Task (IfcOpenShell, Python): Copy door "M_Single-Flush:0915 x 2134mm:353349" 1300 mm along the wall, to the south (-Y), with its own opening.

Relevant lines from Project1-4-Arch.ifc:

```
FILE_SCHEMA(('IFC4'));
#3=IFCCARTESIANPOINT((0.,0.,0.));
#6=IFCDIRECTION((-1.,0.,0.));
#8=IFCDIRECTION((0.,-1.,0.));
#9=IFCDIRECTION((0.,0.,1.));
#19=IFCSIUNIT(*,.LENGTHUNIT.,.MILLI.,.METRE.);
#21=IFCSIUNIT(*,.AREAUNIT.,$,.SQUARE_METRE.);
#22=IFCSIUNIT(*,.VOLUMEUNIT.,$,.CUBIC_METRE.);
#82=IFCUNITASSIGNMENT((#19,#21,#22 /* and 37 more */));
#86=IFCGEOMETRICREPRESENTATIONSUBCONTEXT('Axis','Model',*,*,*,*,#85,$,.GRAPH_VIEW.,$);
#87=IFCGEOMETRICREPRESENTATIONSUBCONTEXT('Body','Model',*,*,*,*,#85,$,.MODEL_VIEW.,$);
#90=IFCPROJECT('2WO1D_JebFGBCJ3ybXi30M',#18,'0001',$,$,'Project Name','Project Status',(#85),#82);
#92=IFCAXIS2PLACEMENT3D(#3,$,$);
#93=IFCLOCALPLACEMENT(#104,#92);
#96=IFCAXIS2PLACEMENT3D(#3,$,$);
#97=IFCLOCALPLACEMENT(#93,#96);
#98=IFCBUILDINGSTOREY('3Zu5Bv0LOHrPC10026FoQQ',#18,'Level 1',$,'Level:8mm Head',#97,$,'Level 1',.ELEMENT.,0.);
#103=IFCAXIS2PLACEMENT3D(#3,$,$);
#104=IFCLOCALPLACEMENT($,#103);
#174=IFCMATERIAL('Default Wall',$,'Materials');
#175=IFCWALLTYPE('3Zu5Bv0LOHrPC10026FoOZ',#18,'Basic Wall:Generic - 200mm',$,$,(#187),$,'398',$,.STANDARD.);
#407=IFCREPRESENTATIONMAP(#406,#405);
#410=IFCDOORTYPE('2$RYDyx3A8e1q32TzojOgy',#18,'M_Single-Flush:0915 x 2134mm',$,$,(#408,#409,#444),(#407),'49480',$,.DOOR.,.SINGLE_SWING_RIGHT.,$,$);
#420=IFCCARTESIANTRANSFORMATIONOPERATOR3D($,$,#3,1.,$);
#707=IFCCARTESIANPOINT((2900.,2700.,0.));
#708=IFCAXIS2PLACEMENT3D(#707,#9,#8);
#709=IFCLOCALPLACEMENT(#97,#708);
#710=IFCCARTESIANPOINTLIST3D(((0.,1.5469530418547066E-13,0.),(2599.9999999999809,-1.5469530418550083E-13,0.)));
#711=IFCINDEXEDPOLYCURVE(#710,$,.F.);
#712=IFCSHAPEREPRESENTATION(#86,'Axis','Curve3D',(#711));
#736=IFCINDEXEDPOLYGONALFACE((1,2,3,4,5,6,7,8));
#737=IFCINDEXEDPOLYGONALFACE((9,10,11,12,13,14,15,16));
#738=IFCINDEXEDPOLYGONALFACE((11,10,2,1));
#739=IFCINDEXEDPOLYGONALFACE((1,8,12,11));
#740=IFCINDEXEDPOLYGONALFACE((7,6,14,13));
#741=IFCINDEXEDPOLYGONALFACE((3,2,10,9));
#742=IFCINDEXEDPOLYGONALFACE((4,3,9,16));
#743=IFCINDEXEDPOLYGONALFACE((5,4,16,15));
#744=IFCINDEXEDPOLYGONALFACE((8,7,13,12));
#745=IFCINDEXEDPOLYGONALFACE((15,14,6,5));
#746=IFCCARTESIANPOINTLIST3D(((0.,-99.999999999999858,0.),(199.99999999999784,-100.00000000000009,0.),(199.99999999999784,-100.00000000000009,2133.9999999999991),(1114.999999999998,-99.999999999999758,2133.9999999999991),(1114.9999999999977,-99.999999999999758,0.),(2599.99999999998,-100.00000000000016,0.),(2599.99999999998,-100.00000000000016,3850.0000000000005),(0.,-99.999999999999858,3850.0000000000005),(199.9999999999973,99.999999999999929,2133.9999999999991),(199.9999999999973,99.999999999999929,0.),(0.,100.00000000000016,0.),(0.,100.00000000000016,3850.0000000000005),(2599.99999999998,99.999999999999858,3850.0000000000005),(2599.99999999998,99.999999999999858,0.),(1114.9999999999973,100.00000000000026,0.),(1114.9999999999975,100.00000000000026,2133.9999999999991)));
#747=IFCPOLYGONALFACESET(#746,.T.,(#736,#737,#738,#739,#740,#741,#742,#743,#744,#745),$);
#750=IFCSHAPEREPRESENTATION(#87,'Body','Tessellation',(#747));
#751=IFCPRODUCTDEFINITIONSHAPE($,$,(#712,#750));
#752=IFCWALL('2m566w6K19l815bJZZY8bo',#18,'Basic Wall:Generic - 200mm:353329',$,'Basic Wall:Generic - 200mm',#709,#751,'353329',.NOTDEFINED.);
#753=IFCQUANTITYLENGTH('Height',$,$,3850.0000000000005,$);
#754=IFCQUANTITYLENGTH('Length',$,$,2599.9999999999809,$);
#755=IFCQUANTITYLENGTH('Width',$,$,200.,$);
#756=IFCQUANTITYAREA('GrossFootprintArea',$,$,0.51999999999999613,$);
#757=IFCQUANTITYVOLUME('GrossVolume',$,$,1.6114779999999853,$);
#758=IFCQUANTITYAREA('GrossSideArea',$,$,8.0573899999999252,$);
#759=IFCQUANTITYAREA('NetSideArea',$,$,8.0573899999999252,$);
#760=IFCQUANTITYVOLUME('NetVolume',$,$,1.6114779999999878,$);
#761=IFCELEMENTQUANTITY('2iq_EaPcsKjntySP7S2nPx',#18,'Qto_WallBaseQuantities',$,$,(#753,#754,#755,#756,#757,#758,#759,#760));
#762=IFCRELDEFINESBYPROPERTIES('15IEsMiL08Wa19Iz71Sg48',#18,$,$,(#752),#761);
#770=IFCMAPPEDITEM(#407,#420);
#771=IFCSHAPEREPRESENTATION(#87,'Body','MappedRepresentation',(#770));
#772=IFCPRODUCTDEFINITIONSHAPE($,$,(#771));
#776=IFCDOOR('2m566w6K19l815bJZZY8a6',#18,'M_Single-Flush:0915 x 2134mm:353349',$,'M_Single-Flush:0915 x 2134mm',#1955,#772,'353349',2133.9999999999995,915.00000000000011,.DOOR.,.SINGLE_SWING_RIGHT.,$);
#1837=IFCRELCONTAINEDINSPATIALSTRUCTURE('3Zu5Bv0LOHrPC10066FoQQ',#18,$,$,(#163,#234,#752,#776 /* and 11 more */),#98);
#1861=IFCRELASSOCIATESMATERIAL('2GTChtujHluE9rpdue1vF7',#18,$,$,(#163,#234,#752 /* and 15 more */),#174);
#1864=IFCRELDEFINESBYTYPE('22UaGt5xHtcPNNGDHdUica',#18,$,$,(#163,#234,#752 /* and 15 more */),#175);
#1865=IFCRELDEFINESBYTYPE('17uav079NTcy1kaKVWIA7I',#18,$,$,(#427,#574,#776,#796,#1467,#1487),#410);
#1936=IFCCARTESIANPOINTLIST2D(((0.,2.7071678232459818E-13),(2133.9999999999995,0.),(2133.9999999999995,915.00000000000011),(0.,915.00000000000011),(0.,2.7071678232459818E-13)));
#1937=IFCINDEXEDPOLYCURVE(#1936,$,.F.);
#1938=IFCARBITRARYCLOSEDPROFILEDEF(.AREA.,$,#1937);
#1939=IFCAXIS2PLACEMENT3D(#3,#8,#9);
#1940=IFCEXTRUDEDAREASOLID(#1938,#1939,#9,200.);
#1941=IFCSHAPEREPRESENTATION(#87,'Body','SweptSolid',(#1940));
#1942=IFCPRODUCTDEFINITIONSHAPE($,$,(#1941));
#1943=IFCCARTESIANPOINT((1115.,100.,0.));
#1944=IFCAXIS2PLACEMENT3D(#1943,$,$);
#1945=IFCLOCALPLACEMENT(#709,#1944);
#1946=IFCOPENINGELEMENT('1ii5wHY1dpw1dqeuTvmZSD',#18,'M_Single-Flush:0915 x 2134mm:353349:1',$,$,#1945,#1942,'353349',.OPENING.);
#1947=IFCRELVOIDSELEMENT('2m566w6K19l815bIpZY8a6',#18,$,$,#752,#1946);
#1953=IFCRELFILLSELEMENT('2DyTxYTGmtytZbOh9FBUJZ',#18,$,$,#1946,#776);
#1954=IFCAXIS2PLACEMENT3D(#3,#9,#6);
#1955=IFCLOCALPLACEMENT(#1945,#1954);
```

```python
import ifcopenshell
import ifcopenshell.api.feature
import ifcopenshell.api.geometry
import ifcopenshell.api.pset
import ifcopenshell.api.root
import ifcopenshell.geom
import ifcopenshell.util.element
import ifcopenshell.util.placement
import ifcopenshell.util.shape
import ifcopenshell.util.unit

model = ifcopenshell.open("Project1-4-Arch.ifc")
area_scale = ifcopenshell.util.unit.calculate_unit_scale(model, "AREAUNIT")
volume_scale = ifcopenshell.util.unit.calculate_unit_scale(model, "VOLUMEUNIT")
settings = ifcopenshell.geom.settings()


def volume(element):
    """Net volume in cubic metres, openings subtracted."""
    shape = ifcopenshell.geom.create_shape(settings, element)
    return ifcopenshell.util.shape.get_volume(shape.geometry)


def reuse_history(source, copy):
    """copy_class also copies each property set's owner history, people and application; keep the originals."""
    for rel in copy.IsDefinedBy:
        if rel.is_a("IfcRelDefinesByProperties") and (history := rel.RelatingPropertyDefinition.OwnerHistory):
            rel.RelatingPropertyDefinition.OwnerHistory = source.OwnerHistory
            ifcopenshell.util.element.remove_deep2(model, history)


door = model.by_id(776)
opening = door.FillsVoids[0].RelatingOpeningElement
wall = opening.VoidsElements[0].RelatingBuildingElement
before = volume(wall)
shift = ifcopenshell.util.placement.get_local_placement(wall.ObjectPlacement)[:3, 0] * 1300.0

# copy_class copies the void relationship, type, container and properties, but no geometry.
new_opening = ifcopenshell.api.root.copy_class(model, product=opening)
new_opening.Representation = ifcopenshell.util.element.copy_deep(
    model, opening.Representation, exclude=["IfcGeometricRepresentationContext", "IfcRepresentationMap"]
)
new_opening.Name = "M_Single-Flush:0915 x 2134mm"
new_opening.Tag = None
reuse_history(opening, new_opening)
new_door = ifcopenshell.api.root.copy_class(model, product=door)
new_door.Representation = ifcopenshell.util.element.copy_deep(
    model, door.Representation, exclude=["IfcGeometricRepresentationContext", "IfcRepresentationMap"]
)
new_door.Name = "M_Single-Flush:0915 x 2134mm"
new_door.Tag = None
reuse_history(door, new_door)
ifcopenshell.api.feature.add_filling(model, opening=new_opening, element=new_door)

for old, new in ((opening, new_opening), (door, new_door)):
    matrix = ifcopenshell.util.placement.get_local_placement(old.ObjectPlacement)
    matrix[:3, 3] += shift
    ifcopenshell.api.geometry.edit_object_placement(model, product=new, matrix=matrix, is_si=False)

after = volume(wall)
thickness = 0.2  # wall thickness in metres

# Update the wall's stored quantities.
qto = model.by_id(ifcopenshell.util.element.get_pset(wall, "Qto_WallBaseQuantities", should_inherit=False)["id"])
ifcopenshell.api.pset.edit_qto(model, qto=qto, properties={
    "NetSideArea": after / thickness / area_scale,
    "NetVolume": after / volume_scale,
})

print(f"wall volume {before:.3f} -> {after:.3f} m3")

model.write("Project1-4-Arch_edited.ifc")
```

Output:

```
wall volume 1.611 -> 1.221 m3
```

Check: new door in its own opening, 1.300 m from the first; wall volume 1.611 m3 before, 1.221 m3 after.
